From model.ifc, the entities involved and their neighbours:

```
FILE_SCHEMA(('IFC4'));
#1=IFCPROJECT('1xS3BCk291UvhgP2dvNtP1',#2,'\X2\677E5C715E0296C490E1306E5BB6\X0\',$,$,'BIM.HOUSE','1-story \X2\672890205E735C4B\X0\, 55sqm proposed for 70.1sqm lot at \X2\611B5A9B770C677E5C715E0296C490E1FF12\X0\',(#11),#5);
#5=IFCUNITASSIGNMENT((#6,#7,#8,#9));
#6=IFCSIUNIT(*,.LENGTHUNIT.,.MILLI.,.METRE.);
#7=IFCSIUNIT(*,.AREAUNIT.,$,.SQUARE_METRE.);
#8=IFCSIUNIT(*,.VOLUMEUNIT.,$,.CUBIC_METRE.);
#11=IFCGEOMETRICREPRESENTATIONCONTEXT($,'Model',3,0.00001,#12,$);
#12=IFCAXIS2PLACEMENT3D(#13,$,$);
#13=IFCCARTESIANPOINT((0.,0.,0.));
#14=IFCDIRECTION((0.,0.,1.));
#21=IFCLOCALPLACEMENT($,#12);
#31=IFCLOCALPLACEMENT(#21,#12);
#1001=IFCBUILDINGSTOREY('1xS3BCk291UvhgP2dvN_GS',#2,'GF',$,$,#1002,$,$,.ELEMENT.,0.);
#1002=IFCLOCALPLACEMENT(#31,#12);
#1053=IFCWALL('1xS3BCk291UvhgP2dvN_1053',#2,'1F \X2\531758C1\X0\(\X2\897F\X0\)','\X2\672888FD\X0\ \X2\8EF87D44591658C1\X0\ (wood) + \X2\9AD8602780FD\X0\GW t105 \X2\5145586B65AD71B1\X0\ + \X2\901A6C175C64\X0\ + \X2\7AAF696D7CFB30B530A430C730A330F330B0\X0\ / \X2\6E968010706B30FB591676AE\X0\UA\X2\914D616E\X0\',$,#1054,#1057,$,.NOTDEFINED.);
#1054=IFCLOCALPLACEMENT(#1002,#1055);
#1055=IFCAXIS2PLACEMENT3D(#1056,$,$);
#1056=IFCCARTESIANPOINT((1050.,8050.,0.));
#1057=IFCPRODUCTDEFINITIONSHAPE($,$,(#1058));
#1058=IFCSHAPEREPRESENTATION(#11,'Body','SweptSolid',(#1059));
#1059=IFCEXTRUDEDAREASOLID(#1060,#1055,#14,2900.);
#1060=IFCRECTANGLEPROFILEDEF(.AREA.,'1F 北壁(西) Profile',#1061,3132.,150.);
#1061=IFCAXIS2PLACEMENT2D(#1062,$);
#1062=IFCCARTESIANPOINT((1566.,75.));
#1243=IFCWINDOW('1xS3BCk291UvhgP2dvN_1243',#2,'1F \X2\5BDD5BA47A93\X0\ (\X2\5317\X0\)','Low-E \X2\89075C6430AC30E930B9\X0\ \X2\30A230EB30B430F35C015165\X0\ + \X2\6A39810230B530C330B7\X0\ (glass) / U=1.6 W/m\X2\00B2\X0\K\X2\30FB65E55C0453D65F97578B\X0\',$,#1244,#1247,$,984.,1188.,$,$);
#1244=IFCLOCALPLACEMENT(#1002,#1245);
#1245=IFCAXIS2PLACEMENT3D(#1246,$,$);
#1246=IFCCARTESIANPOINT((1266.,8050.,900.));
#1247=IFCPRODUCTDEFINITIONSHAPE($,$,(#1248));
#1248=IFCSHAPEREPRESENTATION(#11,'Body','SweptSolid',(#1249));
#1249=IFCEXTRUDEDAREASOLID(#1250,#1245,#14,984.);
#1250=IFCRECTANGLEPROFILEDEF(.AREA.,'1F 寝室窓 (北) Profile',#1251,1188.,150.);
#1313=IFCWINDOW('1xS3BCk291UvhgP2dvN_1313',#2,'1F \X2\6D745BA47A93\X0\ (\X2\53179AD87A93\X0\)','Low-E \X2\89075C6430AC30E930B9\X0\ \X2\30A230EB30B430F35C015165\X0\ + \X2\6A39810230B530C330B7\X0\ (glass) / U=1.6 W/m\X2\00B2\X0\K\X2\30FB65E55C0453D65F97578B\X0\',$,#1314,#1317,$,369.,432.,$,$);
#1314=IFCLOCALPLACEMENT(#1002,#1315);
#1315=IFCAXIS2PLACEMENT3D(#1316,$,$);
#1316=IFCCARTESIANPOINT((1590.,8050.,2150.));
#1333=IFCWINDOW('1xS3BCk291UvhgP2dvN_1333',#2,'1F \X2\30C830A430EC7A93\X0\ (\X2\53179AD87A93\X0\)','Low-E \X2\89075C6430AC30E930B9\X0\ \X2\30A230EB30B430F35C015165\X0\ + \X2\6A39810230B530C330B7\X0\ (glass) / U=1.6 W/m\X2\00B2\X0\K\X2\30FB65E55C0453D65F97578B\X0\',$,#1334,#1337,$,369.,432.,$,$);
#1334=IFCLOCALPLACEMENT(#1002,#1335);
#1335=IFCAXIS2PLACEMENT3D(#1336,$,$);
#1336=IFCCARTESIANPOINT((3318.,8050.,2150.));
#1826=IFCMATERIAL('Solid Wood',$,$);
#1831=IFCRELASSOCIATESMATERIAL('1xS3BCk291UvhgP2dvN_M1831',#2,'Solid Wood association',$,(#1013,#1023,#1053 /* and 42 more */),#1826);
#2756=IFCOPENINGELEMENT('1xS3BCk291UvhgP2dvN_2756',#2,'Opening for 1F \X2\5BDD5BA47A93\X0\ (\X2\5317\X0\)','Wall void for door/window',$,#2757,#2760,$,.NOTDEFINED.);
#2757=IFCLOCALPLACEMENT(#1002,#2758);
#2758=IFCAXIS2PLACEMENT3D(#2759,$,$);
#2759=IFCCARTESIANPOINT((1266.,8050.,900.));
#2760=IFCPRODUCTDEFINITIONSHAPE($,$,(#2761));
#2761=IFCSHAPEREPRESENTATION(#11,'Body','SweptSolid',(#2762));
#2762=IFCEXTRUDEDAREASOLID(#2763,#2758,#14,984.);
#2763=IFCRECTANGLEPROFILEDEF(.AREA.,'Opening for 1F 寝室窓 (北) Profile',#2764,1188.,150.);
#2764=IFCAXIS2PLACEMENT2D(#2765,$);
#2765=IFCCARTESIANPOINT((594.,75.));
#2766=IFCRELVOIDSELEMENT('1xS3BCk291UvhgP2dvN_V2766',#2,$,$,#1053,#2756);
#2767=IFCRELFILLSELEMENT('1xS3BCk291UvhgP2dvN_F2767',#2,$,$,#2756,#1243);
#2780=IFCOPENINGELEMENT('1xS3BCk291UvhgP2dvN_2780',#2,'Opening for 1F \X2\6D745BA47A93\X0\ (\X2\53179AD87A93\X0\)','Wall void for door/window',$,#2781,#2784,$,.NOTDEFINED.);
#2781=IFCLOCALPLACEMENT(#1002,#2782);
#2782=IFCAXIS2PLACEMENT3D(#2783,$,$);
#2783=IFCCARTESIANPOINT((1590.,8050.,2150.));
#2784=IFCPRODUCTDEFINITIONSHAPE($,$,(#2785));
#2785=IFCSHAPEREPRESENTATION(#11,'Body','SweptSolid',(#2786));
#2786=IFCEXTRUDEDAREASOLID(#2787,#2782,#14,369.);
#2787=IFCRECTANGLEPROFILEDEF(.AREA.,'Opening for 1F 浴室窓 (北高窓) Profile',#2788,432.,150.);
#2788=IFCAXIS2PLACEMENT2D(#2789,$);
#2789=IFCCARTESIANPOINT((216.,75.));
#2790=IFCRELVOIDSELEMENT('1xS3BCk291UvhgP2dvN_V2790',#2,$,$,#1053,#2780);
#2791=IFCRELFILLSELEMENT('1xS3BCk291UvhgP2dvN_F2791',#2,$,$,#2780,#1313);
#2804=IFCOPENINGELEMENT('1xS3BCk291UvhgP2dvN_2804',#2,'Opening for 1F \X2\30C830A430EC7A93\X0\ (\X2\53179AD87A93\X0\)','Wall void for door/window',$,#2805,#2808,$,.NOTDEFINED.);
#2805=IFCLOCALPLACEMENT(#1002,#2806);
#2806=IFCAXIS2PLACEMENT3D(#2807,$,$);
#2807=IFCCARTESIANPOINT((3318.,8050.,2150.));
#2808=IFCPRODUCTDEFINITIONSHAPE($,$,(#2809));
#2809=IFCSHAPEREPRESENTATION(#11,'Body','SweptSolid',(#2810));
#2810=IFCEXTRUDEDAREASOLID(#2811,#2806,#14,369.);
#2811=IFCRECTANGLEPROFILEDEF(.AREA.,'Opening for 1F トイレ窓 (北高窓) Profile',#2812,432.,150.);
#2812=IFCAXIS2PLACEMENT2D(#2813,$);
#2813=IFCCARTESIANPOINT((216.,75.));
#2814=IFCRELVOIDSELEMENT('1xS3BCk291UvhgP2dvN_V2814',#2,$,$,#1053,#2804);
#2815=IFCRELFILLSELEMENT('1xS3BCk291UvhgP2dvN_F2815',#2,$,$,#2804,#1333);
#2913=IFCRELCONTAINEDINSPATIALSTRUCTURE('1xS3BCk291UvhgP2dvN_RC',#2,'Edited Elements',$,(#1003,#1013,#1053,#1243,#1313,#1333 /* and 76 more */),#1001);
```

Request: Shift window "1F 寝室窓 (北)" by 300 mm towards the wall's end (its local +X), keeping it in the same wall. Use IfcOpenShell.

```python
import ifcopenshell
import ifcopenshell.api.geometry
import ifcopenshell.util.placement

model = ifcopenshell.open("model.ifc")

window = model.by_guid("1xS3BCk291UvhgP2dvN_1243")
opening = window.FillsVoids[0].RelatingOpeningElement
wall = opening.VoidsElements[0].RelatingBuildingElement

wall_matrix = ifcopenshell.util.placement.get_local_placement(wall.ObjectPlacement)
shift = wall_matrix[:3, 0] * 300.0
before = ifcopenshell.util.placement.get_local_placement(window.ObjectPlacement)[:3, 3].copy()

# The window is not placed relative to its opening, so move both.
for product in (opening, window):
    matrix = ifcopenshell.util.placement.get_local_placement(product.ObjectPlacement)
    matrix[:3, 3] += shift
    ifcopenshell.api.geometry.edit_object_placement(model, product=product, matrix=matrix, is_si=False)

after = ifcopenshell.util.placement.get_local_placement(window.ObjectPlacement)[:3, 3]
print("window moved by", (after - before).round(3) + 0.0)

model.write("model_v2.ifc")
```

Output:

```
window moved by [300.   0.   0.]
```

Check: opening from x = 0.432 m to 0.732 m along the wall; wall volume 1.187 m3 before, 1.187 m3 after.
